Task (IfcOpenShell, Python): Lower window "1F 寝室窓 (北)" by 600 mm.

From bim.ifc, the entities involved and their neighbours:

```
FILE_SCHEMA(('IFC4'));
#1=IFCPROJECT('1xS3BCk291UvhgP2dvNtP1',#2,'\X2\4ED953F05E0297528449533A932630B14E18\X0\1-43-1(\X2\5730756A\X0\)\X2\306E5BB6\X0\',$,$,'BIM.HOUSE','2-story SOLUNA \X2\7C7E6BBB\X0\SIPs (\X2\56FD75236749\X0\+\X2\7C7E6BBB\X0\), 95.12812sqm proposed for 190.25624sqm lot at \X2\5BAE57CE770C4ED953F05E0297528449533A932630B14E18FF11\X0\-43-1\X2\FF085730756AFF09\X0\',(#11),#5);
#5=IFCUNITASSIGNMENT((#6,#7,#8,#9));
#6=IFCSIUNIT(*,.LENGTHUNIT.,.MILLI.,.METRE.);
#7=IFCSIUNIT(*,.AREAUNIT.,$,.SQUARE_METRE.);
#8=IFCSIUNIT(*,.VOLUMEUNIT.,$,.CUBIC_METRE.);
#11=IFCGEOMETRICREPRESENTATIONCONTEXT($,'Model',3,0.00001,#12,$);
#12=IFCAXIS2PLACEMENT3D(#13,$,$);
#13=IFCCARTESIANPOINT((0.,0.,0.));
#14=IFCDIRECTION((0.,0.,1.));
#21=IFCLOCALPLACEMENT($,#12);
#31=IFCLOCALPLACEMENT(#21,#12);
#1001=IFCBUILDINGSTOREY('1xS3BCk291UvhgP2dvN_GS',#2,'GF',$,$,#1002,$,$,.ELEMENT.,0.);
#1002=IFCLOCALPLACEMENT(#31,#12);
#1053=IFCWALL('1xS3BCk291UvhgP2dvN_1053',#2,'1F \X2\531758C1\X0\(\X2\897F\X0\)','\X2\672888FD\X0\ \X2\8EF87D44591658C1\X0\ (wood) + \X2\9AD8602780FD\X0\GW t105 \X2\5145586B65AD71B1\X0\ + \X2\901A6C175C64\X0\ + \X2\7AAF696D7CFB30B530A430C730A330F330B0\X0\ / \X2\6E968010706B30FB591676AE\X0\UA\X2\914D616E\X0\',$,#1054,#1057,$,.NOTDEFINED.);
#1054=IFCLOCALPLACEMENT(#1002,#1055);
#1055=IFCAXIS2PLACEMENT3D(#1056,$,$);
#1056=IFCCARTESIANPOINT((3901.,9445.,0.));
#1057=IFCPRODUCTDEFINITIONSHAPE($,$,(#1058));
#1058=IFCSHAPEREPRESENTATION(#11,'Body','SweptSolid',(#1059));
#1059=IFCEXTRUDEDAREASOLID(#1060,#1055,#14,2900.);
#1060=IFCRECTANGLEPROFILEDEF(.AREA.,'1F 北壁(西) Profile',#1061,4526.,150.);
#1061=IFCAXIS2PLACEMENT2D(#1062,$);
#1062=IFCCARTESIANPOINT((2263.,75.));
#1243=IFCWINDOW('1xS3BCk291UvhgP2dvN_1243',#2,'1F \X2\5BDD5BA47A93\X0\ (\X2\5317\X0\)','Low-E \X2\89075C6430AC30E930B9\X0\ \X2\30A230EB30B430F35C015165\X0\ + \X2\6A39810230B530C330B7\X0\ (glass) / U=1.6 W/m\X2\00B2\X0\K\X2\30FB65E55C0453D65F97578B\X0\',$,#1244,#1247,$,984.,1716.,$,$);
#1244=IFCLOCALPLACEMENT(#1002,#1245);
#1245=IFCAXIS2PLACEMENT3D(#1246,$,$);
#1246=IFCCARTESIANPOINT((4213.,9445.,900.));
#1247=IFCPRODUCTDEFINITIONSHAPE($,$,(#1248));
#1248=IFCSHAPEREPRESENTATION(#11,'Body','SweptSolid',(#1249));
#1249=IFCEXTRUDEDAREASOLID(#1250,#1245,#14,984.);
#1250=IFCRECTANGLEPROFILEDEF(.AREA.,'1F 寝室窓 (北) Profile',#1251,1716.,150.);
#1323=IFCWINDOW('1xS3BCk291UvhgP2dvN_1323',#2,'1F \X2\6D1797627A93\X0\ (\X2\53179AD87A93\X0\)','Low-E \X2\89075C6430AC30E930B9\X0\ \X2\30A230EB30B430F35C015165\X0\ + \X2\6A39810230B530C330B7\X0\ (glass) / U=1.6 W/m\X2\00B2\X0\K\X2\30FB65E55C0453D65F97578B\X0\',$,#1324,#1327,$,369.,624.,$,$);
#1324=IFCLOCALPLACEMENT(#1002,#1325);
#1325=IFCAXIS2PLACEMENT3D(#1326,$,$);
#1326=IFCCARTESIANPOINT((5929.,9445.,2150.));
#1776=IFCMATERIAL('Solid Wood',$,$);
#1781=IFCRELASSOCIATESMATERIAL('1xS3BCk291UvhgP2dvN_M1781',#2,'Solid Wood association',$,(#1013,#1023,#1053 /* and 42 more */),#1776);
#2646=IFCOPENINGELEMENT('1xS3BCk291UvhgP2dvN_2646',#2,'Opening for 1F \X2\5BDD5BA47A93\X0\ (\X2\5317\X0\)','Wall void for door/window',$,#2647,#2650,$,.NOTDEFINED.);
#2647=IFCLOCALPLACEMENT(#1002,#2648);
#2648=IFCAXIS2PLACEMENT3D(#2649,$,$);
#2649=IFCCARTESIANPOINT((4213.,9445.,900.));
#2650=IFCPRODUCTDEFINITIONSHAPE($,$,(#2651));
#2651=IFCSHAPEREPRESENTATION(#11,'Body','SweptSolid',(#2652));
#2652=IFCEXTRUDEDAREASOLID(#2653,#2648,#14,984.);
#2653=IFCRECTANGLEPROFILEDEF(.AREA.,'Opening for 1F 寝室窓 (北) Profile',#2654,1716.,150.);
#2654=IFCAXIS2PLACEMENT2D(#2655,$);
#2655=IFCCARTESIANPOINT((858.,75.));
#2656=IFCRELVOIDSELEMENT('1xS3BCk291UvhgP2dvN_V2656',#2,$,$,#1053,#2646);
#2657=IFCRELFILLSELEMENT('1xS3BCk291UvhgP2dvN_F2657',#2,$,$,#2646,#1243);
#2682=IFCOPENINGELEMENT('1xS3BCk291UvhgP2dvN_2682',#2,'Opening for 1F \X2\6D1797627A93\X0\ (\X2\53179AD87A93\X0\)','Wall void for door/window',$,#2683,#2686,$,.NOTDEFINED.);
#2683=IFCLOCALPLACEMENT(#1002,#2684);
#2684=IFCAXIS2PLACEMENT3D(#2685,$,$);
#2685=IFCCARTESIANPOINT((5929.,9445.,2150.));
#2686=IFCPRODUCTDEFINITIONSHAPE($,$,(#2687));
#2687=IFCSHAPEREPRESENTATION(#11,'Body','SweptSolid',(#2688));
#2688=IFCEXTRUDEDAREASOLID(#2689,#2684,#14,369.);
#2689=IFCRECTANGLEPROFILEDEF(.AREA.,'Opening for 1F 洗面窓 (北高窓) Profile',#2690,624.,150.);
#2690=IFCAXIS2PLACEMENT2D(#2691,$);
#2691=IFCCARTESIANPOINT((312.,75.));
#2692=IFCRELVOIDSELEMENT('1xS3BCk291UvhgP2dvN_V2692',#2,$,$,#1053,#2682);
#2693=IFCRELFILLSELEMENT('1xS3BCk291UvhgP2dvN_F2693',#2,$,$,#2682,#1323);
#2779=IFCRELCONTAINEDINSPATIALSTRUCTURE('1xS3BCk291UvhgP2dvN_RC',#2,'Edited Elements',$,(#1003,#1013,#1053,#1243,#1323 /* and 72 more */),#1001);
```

```python
import numpy as np
import ifcopenshell
import ifcopenshell.api.geometry
import ifcopenshell.util.placement
import ifcopenshell.util.unit

model = ifcopenshell.open("bim.ifc")
unit_scale = ifcopenshell.util.unit.calculate_unit_scale(model)

window = model.by_id(1243)
opening = window.FillsVoids[0].RelatingOpeningElement
dz = -600.0

shift = np.array([0.0, 0.0, dz])
# The window is not placed relative to its opening, so move both.
for product in (opening, window):
    matrix = ifcopenshell.util.placement.get_local_placement(product.ObjectPlacement)
    matrix[:3, 3] += shift
    ifcopenshell.api.geometry.edit_object_placement(model, product=product, matrix=matrix, is_si=False)

print(f"moved by {dz * unit_scale:+.3f} m")

model.write("bim-out.ifc")
```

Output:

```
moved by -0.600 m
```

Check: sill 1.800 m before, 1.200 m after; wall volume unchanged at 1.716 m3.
